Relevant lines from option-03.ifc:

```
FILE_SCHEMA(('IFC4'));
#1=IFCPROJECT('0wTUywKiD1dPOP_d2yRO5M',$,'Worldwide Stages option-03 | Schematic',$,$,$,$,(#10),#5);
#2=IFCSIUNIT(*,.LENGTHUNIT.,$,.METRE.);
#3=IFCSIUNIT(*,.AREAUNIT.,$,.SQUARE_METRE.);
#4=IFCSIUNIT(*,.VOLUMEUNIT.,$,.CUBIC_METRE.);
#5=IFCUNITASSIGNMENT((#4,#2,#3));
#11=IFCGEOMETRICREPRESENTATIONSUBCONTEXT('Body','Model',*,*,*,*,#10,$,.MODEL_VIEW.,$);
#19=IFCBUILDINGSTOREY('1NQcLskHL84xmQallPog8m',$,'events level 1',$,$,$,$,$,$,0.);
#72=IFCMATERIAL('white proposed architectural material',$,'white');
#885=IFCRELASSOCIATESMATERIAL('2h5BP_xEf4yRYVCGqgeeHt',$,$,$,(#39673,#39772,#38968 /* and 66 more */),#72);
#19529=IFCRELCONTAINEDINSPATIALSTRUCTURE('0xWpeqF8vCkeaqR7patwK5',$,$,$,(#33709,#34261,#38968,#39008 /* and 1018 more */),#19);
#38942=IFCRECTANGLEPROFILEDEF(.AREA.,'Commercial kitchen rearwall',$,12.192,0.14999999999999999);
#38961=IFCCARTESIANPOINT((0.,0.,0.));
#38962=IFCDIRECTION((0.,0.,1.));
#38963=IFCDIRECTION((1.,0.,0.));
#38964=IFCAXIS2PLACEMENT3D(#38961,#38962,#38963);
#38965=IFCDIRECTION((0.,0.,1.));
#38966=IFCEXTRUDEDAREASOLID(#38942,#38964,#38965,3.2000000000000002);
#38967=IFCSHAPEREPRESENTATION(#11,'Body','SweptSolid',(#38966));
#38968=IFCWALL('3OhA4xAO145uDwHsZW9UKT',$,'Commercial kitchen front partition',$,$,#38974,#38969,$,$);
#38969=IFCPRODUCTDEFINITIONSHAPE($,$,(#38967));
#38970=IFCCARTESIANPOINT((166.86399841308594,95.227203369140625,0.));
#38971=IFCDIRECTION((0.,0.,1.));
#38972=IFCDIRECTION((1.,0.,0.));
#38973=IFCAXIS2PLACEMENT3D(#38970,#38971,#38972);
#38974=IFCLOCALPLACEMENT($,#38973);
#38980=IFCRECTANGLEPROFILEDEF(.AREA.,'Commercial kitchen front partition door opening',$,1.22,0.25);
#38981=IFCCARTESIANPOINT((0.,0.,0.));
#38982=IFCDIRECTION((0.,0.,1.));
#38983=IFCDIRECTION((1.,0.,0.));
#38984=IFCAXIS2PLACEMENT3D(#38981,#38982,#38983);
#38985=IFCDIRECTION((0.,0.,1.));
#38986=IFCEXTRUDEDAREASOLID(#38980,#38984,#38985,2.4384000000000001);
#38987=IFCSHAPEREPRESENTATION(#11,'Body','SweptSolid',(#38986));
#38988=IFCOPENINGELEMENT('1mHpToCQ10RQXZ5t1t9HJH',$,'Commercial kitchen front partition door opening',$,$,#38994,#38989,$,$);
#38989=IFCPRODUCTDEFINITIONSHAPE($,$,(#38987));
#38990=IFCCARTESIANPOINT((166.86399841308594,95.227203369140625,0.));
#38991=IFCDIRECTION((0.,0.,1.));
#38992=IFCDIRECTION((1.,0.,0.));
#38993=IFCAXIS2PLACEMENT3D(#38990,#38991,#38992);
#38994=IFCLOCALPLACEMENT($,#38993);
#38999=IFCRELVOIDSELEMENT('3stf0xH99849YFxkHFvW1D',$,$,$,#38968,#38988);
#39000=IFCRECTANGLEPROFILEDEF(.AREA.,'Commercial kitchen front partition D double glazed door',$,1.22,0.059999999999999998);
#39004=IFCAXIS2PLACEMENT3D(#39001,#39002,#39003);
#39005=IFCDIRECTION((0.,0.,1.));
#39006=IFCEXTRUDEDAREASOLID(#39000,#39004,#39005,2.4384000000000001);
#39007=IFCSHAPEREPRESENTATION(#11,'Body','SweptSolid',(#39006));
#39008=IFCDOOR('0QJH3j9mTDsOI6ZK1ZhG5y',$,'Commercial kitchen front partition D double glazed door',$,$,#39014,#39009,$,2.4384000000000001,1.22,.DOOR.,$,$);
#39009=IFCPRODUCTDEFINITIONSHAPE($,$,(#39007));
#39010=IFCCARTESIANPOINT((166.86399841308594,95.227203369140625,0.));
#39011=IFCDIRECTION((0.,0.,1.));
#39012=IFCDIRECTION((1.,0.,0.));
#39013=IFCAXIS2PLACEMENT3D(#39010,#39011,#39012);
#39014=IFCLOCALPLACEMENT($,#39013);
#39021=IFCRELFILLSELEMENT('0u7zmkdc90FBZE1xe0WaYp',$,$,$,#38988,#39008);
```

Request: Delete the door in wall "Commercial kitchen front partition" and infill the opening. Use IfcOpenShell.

```python
import ifcopenshell
import ifcopenshell.api.feature
import ifcopenshell.api.root
import ifcopenshell.geom
import ifcopenshell.util.shape

model = ifcopenshell.open("option-03.ifc")
settings = ifcopenshell.geom.settings()


def volume(element):
    """Net volume in cubic metres, openings subtracted."""
    shape = ifcopenshell.geom.create_shape(settings, element)
    return ifcopenshell.util.shape.get_volume(shape.geometry)


door = model.by_guid("0QJH3j9mTDsOI6ZK1ZhG5y")
opening = door.FillsVoids[0].RelatingOpeningElement
wall = opening.VoidsElements[0].RelatingBuildingElement
before = volume(wall)

ifcopenshell.api.root.remove_product(model, product=door)
ifcopenshell.api.feature.remove_feature(model, feature=opening)

after = volume(wall)

print(f"wall volume {before:.3f} -> {after:.3f} m3")

model.write("option-03_edited.ifc")
```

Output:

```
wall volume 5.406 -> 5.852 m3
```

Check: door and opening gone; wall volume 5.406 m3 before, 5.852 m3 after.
